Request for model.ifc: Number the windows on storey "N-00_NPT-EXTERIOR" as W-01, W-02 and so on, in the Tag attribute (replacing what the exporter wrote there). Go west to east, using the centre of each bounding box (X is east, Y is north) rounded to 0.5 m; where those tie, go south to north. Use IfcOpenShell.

First a look at what the model holds.

```python
import ifcopenshell
import ifcopenshell.util.element
import ifcopenshell.util.placement

model = ifcopenshell.open("model.ifc")
print(model.schema)
storey = next(s for s in model.by_type("IfcBuildingStorey") if s.Name == "N-00_NPT-EXTERIOR")
windows = [e for e in ifcopenshell.util.element.get_decomposition(storey) if e.is_a("IfcWindow")]
for e in sorted(windows, key=lambda e: e.id()):
    origin = ifcopenshell.util.placement.get_local_placement(e.ObjectPlacement)[:3, 3]
    print(e.id(), e.Tag, e.Name, origin.round(2) + 0.0, sep=" | ")
```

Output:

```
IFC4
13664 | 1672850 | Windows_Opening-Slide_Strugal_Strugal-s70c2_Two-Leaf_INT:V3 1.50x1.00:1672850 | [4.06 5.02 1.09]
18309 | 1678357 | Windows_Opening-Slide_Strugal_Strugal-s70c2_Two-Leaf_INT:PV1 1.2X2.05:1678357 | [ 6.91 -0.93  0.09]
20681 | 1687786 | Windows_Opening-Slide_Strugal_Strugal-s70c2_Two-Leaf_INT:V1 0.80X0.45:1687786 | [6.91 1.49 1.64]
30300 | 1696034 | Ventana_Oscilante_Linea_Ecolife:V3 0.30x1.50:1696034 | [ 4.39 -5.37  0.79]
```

```python
import ifcopenshell
import ifcopenshell.geom
import ifcopenshell.util.element
import ifcopenshell.util.shape

model = ifcopenshell.open("model.ifc")
settings = ifcopenshell.geom.settings()
settings.set("use-world-coords", True)


def centre(element):
    shape = ifcopenshell.geom.create_shape(settings, element)
    return ifcopenshell.util.shape.get_bbox_centroid(shape.geometry)


storey = next(s for s in model.by_type("IfcBuildingStorey") if s.Name == "N-00_NPT-EXTERIOR")
windows = [e for e in ifcopenshell.util.element.get_decomposition(storey) if e.is_a("IfcWindow")]

# Insertion points can sit at a corner or the storey origin, so sort by the geometry (in metres).
centres = {e: centre(e) for e in windows}
windows.sort(key=lambda e: (round(centres[e][0] / 0.5), centres[e][1]))

for i, e in enumerate(windows, start=1):
    number = f"W-{i:02d}"
    e.Tag = number
    print(e.id(), number)

model.write("model_updated.ifc")
```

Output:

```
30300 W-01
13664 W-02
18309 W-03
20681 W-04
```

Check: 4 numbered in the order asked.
